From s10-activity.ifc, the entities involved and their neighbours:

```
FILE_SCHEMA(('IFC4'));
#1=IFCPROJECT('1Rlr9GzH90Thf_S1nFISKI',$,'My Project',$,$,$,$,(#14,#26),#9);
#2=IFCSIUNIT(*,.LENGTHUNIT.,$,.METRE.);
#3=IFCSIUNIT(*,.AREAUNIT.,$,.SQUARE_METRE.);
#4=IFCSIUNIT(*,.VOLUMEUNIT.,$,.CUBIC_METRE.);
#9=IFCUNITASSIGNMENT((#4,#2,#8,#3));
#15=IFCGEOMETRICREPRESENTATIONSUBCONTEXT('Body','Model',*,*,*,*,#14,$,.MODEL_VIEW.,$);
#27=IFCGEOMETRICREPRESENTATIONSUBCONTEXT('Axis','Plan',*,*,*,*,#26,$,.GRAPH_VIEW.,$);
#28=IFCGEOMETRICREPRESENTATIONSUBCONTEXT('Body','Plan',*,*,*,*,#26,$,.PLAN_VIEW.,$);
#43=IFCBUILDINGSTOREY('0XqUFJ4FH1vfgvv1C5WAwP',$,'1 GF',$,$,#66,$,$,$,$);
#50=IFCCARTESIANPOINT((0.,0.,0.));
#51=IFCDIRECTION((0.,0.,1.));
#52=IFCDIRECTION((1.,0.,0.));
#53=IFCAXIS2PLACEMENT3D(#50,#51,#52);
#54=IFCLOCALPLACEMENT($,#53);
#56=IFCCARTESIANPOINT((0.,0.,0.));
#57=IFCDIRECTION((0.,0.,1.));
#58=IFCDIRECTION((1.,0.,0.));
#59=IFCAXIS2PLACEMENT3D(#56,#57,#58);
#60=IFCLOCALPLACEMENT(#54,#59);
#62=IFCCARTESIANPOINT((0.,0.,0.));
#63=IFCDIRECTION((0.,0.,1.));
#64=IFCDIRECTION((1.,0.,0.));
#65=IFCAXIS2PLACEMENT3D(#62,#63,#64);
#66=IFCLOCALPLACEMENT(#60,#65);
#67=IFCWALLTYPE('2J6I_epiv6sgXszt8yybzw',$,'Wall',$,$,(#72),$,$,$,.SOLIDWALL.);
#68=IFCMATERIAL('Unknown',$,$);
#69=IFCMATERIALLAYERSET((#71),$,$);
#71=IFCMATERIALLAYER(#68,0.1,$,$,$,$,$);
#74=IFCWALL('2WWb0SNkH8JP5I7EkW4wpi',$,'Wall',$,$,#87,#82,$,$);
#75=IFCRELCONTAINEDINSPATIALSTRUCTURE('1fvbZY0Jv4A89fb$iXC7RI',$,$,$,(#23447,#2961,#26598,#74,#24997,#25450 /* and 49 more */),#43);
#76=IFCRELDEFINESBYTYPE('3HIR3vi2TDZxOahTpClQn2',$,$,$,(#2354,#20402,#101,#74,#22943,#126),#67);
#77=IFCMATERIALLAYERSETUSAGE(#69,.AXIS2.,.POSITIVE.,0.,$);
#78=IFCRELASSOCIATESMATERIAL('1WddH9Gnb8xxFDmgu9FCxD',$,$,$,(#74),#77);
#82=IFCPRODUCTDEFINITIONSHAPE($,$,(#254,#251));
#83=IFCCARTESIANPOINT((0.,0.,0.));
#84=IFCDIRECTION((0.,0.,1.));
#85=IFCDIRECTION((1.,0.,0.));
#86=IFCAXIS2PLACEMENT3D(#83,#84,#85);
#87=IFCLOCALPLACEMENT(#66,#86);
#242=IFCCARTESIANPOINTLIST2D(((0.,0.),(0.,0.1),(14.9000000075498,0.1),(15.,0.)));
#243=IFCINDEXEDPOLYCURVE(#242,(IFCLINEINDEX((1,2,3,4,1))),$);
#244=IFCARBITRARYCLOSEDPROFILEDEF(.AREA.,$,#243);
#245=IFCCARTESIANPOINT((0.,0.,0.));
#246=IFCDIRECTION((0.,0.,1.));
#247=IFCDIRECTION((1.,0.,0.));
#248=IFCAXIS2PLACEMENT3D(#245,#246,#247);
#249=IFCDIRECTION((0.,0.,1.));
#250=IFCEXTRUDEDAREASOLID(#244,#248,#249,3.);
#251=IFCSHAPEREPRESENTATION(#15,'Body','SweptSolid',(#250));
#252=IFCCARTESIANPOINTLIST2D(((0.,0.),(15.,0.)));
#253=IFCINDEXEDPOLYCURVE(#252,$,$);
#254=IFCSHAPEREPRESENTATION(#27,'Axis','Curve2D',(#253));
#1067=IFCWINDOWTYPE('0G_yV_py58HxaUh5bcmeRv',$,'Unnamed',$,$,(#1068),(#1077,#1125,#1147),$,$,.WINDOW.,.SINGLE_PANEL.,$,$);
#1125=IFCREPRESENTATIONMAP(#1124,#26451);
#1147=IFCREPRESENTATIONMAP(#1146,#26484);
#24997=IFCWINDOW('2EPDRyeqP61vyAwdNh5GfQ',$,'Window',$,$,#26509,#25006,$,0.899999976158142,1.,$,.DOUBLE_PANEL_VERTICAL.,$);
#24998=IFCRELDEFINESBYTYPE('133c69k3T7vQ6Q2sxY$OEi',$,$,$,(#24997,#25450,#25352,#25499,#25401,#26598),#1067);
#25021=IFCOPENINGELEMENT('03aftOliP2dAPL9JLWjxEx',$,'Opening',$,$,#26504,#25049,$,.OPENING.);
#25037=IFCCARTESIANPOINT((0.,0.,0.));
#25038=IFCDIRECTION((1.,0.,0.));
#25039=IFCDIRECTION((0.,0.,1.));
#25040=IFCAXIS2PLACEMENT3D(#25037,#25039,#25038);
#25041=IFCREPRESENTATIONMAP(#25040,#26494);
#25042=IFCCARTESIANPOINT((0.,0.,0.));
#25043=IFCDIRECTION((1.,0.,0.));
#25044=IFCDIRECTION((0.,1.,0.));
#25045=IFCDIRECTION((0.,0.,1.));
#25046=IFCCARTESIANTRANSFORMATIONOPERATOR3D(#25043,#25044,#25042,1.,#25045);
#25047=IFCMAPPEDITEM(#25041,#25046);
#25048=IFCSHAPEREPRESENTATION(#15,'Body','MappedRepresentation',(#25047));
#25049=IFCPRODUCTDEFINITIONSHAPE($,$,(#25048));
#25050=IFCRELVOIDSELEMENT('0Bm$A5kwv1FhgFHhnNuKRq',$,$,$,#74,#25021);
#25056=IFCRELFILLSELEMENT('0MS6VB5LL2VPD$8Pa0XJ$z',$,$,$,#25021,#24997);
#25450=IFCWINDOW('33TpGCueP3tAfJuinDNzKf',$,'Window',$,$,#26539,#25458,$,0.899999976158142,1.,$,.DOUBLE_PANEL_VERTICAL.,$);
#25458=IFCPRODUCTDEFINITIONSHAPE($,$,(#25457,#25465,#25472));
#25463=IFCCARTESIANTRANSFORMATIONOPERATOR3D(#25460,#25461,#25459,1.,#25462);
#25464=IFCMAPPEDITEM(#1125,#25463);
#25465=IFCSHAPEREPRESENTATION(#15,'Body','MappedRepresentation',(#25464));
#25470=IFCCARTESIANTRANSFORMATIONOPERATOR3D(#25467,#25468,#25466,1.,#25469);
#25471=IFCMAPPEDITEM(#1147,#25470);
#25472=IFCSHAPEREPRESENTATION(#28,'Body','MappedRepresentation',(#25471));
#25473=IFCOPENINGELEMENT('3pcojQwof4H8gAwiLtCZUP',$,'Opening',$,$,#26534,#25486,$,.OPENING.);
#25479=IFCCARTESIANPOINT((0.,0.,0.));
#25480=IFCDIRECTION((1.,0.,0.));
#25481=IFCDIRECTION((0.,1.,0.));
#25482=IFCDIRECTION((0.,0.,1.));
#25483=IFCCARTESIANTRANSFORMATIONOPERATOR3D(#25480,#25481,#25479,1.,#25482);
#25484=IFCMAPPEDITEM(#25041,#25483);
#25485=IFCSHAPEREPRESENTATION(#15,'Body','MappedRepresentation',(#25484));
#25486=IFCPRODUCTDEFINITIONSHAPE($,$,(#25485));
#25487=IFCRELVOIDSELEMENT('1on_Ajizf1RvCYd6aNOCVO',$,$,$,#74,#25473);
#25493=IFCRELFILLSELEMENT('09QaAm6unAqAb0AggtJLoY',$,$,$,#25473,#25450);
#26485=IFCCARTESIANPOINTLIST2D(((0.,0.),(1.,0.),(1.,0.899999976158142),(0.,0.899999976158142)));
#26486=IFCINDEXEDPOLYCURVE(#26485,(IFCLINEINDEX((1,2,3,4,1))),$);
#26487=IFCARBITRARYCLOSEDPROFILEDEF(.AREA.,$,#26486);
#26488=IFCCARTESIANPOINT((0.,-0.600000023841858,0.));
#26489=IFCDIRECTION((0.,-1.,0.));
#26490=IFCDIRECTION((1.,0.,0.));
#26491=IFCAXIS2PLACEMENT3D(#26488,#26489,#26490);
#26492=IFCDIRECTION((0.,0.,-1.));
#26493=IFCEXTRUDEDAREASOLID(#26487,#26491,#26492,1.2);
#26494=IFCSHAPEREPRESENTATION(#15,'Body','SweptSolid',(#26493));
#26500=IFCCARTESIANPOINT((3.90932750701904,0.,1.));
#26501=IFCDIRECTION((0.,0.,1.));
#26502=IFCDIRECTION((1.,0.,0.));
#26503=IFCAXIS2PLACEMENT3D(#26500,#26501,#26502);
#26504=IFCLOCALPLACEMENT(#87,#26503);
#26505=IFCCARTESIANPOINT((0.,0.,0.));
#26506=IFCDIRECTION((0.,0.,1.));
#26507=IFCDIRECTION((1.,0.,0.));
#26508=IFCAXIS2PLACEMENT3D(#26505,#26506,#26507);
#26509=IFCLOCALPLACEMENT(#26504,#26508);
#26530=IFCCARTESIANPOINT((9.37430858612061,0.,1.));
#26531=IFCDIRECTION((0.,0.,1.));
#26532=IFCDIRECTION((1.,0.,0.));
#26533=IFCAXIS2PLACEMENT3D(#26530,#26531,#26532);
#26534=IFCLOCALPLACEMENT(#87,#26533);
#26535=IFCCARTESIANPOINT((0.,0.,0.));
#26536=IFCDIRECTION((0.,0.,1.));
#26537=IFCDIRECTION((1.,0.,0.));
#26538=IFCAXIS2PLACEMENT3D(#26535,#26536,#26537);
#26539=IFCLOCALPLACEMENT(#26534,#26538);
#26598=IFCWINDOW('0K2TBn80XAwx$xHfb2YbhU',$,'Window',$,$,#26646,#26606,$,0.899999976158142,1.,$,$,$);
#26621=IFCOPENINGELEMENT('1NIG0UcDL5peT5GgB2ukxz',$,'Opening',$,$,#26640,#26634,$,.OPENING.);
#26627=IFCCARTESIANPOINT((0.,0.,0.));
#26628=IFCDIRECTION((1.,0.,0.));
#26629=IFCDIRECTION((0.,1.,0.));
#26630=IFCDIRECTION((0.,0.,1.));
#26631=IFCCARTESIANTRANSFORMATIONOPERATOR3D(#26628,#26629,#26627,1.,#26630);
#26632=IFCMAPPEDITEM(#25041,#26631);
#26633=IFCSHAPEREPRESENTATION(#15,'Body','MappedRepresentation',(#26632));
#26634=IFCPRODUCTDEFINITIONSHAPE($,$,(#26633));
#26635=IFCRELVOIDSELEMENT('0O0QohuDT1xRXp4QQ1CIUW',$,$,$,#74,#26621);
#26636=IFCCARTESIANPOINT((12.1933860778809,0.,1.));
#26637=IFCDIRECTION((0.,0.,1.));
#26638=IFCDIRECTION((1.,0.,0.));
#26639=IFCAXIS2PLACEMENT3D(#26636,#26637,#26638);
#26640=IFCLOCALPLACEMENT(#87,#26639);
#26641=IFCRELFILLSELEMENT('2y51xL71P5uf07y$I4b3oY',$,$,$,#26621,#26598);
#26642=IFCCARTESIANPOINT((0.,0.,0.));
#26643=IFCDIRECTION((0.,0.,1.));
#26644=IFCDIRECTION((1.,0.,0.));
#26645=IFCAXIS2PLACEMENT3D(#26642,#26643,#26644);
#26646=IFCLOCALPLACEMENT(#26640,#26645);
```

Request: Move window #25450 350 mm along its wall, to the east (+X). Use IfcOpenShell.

```python
import ifcopenshell
import ifcopenshell.api.geometry
import ifcopenshell.util.placement
import ifcopenshell.util.unit

model = ifcopenshell.open("s10-activity.ifc")
unit_scale = ifcopenshell.util.unit.calculate_unit_scale(model)

window = model.by_id(25450)
opening = window.FillsVoids[0].RelatingOpeningElement
wall = opening.VoidsElements[0].RelatingBuildingElement

wall_matrix = ifcopenshell.util.placement.get_local_placement(wall.ObjectPlacement)
shift = wall_matrix[:3, 0] * 0.35 / unit_scale
before = ifcopenshell.util.placement.get_local_placement(window.ObjectPlacement)[:3, 3].copy()

# The window is placed relative to its opening, so it follows when the opening moves.
matrix = ifcopenshell.util.placement.get_local_placement(opening.ObjectPlacement)
matrix[:3, 3] += shift
ifcopenshell.api.geometry.edit_object_placement(
    model, product=opening, matrix=matrix, is_si=False, should_transform_children=True
)

after = ifcopenshell.util.placement.get_local_placement(window.ObjectPlacement)[:3, 3]
print("window moved by", (after - before).round(3) + 0.0)

model.write("s10-activity_updated.ifc")
```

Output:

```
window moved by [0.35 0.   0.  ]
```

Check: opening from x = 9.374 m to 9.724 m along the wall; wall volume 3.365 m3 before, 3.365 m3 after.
